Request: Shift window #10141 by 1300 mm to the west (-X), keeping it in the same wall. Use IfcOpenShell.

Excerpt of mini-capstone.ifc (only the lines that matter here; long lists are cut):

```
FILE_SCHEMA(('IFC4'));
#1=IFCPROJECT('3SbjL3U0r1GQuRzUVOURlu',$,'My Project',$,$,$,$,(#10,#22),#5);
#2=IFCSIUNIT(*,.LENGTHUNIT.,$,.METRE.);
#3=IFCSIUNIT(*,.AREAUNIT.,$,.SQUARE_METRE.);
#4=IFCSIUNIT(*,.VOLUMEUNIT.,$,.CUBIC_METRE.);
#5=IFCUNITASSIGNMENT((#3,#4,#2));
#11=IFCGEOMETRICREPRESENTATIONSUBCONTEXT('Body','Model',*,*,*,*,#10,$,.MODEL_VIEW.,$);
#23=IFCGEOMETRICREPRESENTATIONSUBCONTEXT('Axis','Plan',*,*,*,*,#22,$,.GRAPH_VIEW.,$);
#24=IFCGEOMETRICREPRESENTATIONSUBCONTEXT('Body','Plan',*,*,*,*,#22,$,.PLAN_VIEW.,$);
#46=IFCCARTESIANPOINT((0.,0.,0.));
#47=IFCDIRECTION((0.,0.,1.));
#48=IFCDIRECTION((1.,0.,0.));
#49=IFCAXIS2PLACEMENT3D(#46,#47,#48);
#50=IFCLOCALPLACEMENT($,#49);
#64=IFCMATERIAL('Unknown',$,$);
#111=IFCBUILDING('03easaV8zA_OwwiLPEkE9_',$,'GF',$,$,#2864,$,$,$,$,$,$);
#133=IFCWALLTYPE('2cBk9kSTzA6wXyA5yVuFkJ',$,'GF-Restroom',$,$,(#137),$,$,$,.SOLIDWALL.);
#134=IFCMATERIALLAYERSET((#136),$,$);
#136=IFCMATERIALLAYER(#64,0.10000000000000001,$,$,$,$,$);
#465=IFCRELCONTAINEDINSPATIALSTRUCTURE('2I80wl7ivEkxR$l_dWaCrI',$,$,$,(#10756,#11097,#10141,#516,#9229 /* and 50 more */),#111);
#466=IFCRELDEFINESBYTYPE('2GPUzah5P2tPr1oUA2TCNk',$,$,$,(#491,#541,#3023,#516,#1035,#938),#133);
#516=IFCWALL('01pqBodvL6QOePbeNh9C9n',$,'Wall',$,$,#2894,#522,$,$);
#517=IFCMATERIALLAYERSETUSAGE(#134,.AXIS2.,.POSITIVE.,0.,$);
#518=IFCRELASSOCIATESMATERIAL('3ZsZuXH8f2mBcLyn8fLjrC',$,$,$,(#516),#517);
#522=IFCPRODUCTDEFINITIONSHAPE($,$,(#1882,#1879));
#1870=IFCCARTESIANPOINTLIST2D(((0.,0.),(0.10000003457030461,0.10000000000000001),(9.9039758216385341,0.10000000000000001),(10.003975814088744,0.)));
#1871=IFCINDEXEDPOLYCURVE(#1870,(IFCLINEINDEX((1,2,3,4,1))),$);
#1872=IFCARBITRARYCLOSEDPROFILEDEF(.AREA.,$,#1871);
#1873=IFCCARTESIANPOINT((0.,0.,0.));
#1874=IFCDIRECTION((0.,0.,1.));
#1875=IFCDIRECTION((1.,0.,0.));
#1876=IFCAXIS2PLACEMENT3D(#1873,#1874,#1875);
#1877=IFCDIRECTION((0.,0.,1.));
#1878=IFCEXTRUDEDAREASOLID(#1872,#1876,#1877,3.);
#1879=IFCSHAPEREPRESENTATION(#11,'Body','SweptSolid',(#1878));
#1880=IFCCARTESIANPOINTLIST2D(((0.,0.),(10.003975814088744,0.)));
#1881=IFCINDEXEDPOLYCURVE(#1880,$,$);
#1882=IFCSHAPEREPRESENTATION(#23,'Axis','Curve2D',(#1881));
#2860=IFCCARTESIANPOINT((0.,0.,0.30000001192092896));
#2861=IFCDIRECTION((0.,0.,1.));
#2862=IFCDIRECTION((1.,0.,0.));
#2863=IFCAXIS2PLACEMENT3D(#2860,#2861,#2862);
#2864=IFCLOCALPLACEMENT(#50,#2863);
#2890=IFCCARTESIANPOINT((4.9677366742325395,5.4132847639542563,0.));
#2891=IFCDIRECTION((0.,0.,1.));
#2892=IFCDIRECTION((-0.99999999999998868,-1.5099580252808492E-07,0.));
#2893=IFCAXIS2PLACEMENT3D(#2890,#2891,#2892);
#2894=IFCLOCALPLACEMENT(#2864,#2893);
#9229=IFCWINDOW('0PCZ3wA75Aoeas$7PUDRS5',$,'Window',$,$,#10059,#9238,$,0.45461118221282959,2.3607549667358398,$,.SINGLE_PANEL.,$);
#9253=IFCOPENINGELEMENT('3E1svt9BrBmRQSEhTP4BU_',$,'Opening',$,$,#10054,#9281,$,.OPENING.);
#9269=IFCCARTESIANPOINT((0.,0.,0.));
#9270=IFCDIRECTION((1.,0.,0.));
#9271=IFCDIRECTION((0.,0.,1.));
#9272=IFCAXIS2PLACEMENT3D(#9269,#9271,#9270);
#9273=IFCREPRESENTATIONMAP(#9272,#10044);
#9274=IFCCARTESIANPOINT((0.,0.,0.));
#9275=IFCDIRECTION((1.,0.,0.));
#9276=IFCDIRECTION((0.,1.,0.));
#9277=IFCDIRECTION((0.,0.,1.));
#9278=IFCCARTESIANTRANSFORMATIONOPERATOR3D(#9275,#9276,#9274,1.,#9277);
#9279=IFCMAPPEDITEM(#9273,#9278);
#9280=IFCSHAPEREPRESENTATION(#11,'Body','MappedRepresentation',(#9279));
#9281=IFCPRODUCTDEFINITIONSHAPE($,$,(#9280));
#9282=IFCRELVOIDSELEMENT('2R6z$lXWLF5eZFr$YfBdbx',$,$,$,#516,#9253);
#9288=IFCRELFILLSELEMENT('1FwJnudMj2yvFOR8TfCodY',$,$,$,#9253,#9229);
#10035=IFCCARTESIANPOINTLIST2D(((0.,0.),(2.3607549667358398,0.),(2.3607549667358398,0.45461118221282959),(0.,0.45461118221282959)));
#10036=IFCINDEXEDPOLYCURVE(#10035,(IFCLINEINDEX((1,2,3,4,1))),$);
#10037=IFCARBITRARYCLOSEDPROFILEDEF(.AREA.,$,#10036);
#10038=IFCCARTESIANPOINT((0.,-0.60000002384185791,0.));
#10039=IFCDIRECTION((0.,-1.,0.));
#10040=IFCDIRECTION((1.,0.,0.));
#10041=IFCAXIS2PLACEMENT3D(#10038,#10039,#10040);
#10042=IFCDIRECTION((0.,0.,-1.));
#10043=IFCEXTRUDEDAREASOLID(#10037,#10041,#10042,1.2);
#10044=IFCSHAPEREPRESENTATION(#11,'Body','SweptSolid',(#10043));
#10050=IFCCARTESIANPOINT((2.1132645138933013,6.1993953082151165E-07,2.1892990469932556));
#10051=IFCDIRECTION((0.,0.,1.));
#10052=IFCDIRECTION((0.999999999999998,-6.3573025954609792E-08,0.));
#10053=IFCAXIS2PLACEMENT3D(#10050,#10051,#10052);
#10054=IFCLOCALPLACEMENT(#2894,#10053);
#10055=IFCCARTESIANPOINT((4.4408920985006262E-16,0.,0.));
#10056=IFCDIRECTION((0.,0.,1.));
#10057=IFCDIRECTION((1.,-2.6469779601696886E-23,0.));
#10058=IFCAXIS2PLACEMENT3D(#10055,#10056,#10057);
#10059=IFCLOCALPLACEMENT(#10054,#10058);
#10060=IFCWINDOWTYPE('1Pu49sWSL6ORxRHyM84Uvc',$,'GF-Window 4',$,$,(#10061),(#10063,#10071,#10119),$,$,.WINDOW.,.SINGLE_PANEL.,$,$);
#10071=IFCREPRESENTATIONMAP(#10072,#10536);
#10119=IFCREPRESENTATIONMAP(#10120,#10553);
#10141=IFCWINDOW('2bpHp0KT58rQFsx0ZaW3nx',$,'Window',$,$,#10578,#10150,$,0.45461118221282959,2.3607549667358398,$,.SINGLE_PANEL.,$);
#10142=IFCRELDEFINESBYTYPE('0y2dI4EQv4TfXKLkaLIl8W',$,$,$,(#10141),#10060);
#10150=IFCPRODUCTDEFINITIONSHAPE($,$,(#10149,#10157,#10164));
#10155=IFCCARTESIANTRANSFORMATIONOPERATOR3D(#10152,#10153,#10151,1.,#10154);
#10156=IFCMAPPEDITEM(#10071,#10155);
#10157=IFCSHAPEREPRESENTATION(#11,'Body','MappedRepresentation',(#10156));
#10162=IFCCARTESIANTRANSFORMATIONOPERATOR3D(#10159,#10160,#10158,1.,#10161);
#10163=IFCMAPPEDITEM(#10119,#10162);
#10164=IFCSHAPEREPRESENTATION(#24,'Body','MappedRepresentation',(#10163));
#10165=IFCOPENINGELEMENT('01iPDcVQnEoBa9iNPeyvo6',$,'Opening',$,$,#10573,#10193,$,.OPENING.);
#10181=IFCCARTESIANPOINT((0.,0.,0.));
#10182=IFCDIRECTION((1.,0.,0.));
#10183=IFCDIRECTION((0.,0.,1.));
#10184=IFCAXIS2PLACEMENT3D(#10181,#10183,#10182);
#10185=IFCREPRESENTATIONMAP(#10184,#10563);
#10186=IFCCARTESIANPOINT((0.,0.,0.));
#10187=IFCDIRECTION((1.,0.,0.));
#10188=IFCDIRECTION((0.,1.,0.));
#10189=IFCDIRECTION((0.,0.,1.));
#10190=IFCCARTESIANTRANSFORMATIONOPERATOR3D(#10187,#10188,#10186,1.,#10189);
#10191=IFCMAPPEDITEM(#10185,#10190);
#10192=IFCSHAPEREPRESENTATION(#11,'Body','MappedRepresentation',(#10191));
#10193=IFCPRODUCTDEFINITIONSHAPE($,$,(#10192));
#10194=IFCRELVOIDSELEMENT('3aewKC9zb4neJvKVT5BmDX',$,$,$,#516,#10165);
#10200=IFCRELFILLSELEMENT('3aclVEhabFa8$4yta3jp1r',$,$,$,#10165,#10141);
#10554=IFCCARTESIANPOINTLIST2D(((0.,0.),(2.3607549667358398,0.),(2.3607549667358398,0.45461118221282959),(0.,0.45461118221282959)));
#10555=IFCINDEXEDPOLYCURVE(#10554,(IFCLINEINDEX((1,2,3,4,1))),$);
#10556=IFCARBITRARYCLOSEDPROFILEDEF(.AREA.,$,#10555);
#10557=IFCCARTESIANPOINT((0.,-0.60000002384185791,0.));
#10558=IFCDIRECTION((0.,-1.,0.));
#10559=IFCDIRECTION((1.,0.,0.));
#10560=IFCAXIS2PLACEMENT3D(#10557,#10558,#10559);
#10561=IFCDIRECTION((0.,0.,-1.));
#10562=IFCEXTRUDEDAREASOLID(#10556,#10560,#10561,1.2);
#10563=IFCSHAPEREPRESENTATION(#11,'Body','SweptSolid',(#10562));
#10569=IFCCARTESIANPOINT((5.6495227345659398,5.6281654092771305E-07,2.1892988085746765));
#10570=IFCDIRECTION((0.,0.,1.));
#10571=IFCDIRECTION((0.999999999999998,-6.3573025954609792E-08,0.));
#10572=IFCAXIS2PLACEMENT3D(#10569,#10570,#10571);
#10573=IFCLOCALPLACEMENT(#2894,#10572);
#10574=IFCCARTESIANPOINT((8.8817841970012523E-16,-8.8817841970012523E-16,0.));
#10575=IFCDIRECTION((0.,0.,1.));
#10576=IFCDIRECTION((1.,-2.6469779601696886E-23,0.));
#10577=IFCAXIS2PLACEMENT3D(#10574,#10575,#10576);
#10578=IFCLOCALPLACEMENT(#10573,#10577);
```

```python
import ifcopenshell
import ifcopenshell.api.geometry
import ifcopenshell.util.placement
import ifcopenshell.util.unit

model = ifcopenshell.open("mini-capstone.ifc")
unit_scale = ifcopenshell.util.unit.calculate_unit_scale(model)

window = model.by_guid("2bpHp0KT58rQFsx0ZaW3nx")
opening = window.FillsVoids[0].RelatingOpeningElement
wall = opening.VoidsElements[0].RelatingBuildingElement

wall_matrix = ifcopenshell.util.placement.get_local_placement(wall.ObjectPlacement)
shift = wall_matrix[:3, 0] * 1.3 / unit_scale
before = ifcopenshell.util.placement.get_local_placement(window.ObjectPlacement)[:3, 3].copy()

# The window is placed relative to its opening, so it follows when the opening moves.
matrix = ifcopenshell.util.placement.get_local_placement(opening.ObjectPlacement)
matrix[:3, 3] += shift
ifcopenshell.api.geometry.edit_object_placement(
    model, product=opening, matrix=matrix, is_si=False, should_transform_children=True
)

after = ifcopenshell.util.placement.get_local_placement(window.ObjectPlacement)[:3, 3]
print("window moved by", (after - before).round(3) + 0.0)

model.write("mini-capstone_edited.ifc")
```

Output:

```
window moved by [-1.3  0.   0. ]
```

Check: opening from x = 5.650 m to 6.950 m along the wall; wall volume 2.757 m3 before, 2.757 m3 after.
